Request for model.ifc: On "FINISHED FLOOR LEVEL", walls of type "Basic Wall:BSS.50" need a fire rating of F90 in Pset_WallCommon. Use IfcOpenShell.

First a look at what the model holds.

```python
import ifcopenshell
import ifcopenshell.util.element

model = ifcopenshell.open("model.ifc")
print(model.schema)
storey = next(s for s in model.by_type("IfcBuildingStorey") if s.Name == "FINISHED FLOOR LEVEL")
walls = [e for e in ifcopenshell.util.element.get_decomposition(storey) if e.is_a("IfcWall")]
seen = {}
for e in walls:
    element_type = ifcopenshell.util.element.get_type(e)
    key = (element_type.Name if element_type != e and element_type else None, ifcopenshell.util.element.get_pset(e, "Pset_WallCommon", "FireRating"))
    seen[key] = seen.get(key, 0) + 1
for (name, value), count in sorted(seen.items(), key=str):
    print(count, "x", name, "|", value)
```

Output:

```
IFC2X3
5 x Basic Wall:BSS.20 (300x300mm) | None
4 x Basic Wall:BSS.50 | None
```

```python
import ifcopenshell
import ifcopenshell.api.pset
import ifcopenshell.util.element

model = ifcopenshell.open("model.ifc")

storey = next(s for s in model.by_type("IfcBuildingStorey") if s.Name == "FINISHED FLOOR LEVEL")
walls = [e for e in ifcopenshell.util.element.get_decomposition(storey) if e.is_a("IfcWall")]

count = 0
for e in walls:
    element_type = ifcopenshell.util.element.get_type(e)
    if element_type in (None, e) or element_type.Name != "Basic Wall:BSS.50":
        continue
    # add_pset returns the element's existing set when there is one.
    pset = ifcopenshell.api.pset.add_pset(model, product=e, name="Pset_WallCommon")
    ifcopenshell.api.pset.edit_pset(model, pset=pset, properties={"FireRating": "F90"})
    count += 1

print(count, "walls updated")

model.write("model-out.ifc")
```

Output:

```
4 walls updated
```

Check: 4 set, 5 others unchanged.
